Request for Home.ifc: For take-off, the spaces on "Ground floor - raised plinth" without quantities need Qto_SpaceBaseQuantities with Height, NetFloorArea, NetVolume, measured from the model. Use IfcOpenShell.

First a look at what the model holds.

```python
import ifcopenshell
import ifcopenshell.util.element
import ifcopenshell.util.unit

model = ifcopenshell.open("Home.ifc")
print(model.schema)
for unit_type in ("LENGTHUNIT", "AREAUNIT", "VOLUMEUNIT"):
    print(unit_type, ifcopenshell.util.unit.calculate_unit_scale(model, unit_type))
storey = next(s for s in model.by_type("IfcBuildingStorey") if s.Name == "Ground floor - raised plinth")
spaces = [e for e in ifcopenshell.util.element.get_decomposition(storey) if e.is_a("IfcSpace")]
for e in sorted(spaces, key=lambda e: e.id()):
    print(e.id(), e.is_a(), e.Name, list(ifcopenshell.util.element.get_psets(e, qtos_only=True)), sep=" | ")
```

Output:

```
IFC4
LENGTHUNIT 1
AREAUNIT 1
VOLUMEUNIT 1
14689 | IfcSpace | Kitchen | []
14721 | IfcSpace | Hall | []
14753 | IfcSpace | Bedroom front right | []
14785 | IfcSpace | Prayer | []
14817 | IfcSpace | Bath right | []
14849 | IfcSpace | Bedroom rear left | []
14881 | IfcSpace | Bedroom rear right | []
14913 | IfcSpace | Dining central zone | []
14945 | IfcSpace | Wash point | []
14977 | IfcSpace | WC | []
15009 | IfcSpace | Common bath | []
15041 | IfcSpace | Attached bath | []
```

```python
import ifcopenshell
import ifcopenshell.api.pset
import ifcopenshell.geom
import ifcopenshell.util.element
import ifcopenshell.util.shape
import ifcopenshell.util.unit

model = ifcopenshell.open("Home.ifc")
unit_scale = ifcopenshell.util.unit.calculate_unit_scale(model)
area_scale = ifcopenshell.util.unit.calculate_unit_scale(model, "AREAUNIT")
volume_scale = ifcopenshell.util.unit.calculate_unit_scale(model, "VOLUMEUNIT")
settings = ifcopenshell.geom.settings()

storey = next(s for s in model.by_type("IfcBuildingStorey") if s.Name == "Ground floor - raised plinth")
spaces = [e for e in ifcopenshell.util.element.get_decomposition(storey) if e.is_a("IfcSpace")]

for e in sorted(spaces, key=lambda e: e.id()):
    if ifcopenshell.util.element.get_psets(e, qtos_only=True, should_inherit=False):
        continue
    # Geometry comes back in metres, in the element's own axes.
    shape = ifcopenshell.geom.create_shape(settings, e)
    values = {
        "Height": ifcopenshell.util.shape.get_z(shape.geometry) / unit_scale,
        "NetFloorArea": ifcopenshell.util.shape.get_footprint_area(shape.geometry) / area_scale,
        "NetVolume": ifcopenshell.util.shape.get_volume(shape.geometry) / volume_scale,
    }
    qto = ifcopenshell.api.pset.add_qto(model, product=e, name="Qto_SpaceBaseQuantities")
    ifcopenshell.api.pset.edit_qto(model, qto=qto, properties=values)
    print(e.id(), {k: round(v, 3) for k, v in values.items()})

model.write("Home_edited.ifc")
```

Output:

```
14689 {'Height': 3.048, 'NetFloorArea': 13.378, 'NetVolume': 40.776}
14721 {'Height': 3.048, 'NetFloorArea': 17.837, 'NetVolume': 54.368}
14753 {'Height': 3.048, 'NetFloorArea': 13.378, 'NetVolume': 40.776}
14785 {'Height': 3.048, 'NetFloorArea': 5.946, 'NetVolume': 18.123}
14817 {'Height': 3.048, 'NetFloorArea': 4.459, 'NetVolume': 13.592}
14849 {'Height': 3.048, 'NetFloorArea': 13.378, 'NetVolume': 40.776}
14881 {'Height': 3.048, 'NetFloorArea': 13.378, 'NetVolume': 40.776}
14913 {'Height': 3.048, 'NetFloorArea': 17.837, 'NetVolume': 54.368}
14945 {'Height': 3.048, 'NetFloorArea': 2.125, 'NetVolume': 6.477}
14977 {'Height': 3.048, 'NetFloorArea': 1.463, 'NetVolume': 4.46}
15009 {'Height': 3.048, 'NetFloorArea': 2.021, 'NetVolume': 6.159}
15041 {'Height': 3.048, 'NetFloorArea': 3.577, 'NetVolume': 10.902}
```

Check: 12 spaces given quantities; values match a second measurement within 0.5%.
